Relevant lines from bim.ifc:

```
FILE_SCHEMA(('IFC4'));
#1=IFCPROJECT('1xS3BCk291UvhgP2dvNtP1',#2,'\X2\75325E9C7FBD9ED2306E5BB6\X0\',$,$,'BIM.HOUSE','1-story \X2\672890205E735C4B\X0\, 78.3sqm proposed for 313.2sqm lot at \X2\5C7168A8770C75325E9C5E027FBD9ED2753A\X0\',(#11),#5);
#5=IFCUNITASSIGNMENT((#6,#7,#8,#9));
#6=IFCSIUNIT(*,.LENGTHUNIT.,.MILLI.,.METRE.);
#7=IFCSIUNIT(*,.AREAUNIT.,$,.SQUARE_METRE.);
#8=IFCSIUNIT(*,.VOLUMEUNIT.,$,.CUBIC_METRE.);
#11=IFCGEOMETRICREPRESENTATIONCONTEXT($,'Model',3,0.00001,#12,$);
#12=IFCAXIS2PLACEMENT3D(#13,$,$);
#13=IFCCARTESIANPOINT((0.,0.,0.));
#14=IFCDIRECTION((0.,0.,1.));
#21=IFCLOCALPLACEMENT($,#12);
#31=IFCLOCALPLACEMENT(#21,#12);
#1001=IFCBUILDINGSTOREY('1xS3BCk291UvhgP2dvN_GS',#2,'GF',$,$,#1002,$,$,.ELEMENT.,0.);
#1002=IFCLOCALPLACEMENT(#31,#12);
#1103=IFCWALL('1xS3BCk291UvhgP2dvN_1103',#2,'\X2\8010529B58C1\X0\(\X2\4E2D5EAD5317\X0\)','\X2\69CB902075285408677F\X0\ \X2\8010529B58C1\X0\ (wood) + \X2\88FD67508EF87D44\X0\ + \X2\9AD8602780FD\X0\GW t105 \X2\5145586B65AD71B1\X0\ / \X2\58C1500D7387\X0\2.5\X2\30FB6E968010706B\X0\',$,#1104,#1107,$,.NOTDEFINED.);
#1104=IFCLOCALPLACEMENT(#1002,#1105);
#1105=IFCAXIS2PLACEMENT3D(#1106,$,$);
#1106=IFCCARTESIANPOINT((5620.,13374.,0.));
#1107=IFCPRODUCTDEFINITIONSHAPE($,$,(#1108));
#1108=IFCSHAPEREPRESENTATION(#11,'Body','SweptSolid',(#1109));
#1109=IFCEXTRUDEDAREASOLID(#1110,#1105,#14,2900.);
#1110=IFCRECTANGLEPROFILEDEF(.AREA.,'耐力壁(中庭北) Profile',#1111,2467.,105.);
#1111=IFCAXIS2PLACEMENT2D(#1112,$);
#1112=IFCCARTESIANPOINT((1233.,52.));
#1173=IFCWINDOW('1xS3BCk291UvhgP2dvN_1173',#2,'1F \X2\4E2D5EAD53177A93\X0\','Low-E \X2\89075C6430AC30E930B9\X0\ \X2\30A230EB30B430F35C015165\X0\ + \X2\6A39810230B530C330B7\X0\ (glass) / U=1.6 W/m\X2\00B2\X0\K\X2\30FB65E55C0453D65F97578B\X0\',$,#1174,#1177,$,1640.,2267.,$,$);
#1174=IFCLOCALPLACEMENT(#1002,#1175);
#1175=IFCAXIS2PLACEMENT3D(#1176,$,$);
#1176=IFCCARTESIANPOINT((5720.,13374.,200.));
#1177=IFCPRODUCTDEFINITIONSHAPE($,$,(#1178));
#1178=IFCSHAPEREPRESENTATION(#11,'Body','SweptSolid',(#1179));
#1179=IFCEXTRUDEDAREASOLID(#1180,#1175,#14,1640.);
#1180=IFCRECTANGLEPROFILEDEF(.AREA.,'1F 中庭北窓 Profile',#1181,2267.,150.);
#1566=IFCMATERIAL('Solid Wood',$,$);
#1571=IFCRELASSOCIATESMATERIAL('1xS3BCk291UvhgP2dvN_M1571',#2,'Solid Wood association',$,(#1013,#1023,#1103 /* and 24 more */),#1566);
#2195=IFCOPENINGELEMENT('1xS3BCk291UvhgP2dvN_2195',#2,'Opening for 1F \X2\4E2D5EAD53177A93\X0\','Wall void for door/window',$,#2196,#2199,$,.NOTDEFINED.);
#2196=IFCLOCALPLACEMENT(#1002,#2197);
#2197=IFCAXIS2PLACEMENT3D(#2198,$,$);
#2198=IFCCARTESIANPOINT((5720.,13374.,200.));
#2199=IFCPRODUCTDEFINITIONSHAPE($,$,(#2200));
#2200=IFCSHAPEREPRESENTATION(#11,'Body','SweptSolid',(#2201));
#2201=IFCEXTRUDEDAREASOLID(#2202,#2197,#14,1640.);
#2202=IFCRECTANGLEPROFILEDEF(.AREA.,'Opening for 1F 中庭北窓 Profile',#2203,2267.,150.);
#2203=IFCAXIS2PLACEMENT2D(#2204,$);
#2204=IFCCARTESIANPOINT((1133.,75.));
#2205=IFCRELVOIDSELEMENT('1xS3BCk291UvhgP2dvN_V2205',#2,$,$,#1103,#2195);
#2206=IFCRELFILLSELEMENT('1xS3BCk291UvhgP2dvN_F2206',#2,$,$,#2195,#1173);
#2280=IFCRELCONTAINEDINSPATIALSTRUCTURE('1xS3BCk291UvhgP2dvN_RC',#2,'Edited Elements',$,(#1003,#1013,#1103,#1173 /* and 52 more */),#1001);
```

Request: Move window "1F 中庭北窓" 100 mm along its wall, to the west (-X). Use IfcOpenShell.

```python
import ifcopenshell
import ifcopenshell.api.geometry
import ifcopenshell.util.placement
import ifcopenshell.util.unit

model = ifcopenshell.open("bim.ifc")
unit_scale = ifcopenshell.util.unit.calculate_unit_scale(model)

window = model.by_guid("1xS3BCk291UvhgP2dvN_1173")
opening = window.FillsVoids[0].RelatingOpeningElement
wall = opening.VoidsElements[0].RelatingBuildingElement

wall_matrix = ifcopenshell.util.placement.get_local_placement(wall.ObjectPlacement)
shift = wall_matrix[:3, 0] * -0.1 / unit_scale
before = ifcopenshell.util.placement.get_local_placement(window.ObjectPlacement)[:3, 3].copy()

# The window is not placed relative to its opening, so move both.
for product in (opening, window):
    matrix = ifcopenshell.util.placement.get_local_placement(product.ObjectPlacement)
    matrix[:3, 3] += shift
    ifcopenshell.api.geometry.edit_object_placement(model, product=product, matrix=matrix, is_si=False)

after = ifcopenshell.util.placement.get_local_placement(window.ObjectPlacement)[:3, 3]
print("window moved by", (after - before).round(3) + 0.0)

model.write("bim_edited.ifc")
```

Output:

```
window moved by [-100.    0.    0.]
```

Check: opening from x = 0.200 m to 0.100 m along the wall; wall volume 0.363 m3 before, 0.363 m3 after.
